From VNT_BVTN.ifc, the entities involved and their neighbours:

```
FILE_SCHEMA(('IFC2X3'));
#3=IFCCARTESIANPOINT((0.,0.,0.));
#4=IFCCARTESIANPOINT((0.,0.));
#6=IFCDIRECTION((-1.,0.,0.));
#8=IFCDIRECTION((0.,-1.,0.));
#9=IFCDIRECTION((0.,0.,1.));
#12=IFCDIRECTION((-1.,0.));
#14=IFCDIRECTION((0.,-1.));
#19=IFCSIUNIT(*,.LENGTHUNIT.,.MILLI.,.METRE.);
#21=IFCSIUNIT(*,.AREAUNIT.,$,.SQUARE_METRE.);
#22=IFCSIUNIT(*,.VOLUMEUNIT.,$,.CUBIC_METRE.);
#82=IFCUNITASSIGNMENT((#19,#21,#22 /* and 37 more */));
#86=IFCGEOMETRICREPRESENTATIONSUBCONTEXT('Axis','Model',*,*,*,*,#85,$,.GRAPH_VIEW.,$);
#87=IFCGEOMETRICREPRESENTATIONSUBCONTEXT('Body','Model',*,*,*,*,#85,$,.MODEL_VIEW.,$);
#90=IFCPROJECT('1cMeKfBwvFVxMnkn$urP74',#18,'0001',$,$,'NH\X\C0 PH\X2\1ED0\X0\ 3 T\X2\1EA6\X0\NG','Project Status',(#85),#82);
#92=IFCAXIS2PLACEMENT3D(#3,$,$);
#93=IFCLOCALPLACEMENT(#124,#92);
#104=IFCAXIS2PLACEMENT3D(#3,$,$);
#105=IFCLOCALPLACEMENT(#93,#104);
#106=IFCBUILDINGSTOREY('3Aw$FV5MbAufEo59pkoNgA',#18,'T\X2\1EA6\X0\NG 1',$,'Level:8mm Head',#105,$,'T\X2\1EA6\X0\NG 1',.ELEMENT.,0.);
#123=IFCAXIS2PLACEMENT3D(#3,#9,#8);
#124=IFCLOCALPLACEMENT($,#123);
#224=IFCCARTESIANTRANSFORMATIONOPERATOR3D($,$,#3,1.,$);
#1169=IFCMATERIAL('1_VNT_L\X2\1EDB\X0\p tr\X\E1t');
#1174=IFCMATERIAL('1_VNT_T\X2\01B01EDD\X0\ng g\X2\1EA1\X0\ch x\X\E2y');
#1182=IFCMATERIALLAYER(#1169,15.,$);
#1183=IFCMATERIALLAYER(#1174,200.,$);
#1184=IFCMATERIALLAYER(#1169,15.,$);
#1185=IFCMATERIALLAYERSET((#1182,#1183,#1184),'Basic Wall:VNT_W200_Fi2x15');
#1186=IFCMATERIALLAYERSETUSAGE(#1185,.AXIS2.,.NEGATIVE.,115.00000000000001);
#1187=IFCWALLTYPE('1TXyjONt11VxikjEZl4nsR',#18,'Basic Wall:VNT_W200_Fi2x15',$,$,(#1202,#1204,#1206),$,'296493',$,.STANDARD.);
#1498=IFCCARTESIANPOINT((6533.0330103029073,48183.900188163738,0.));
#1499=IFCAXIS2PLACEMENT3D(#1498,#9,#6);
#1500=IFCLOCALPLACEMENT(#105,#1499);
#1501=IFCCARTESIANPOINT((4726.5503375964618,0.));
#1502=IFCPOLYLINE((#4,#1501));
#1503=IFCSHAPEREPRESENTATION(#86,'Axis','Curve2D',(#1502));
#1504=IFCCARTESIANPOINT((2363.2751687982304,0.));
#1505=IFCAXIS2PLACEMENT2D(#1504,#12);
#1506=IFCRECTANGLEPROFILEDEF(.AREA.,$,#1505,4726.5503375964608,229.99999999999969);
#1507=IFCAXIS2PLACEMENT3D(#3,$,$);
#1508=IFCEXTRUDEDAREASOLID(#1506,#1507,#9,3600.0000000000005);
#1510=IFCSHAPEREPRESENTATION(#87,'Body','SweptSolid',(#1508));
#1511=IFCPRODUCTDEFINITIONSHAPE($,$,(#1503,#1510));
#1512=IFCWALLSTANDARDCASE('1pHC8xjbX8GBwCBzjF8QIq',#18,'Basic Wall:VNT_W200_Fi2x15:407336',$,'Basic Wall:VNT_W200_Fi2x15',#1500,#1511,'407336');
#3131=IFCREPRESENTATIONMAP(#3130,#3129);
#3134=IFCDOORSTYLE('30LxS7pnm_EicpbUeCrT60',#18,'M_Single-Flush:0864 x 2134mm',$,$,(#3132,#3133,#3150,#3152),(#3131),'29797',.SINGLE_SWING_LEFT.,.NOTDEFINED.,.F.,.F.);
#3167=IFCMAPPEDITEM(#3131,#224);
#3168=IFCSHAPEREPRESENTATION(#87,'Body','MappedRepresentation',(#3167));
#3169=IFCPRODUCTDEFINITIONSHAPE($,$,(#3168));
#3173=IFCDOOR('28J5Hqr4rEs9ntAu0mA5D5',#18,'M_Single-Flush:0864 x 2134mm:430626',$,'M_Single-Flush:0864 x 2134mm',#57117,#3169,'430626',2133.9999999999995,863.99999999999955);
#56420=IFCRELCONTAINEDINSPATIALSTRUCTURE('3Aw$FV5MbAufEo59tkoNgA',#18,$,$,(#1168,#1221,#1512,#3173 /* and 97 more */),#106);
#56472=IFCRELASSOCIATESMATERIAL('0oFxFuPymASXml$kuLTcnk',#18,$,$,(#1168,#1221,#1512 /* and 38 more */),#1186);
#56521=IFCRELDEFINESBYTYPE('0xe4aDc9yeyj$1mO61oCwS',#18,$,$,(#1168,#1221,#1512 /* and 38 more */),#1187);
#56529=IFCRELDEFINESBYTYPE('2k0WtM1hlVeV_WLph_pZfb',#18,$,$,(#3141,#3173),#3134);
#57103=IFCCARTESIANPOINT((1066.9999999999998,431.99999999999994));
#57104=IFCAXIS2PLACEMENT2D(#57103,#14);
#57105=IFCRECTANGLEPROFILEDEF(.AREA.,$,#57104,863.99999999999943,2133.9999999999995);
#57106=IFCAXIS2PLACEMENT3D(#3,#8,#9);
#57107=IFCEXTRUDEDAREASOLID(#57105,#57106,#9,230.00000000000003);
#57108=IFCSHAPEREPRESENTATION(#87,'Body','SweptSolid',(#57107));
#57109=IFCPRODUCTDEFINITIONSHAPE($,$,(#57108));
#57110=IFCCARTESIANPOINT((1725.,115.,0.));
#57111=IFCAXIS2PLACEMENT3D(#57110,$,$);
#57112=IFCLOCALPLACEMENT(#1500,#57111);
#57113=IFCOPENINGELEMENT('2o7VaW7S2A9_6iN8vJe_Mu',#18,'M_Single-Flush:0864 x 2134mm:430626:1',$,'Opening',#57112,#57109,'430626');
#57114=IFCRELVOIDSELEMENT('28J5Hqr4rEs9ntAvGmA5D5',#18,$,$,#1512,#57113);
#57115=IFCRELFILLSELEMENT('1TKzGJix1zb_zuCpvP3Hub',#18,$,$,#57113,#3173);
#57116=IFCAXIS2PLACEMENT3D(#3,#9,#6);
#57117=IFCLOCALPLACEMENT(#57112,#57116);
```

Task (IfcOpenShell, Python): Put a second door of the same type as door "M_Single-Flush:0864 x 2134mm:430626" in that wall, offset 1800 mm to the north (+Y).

```python
import ifcopenshell
import ifcopenshell.api.feature
import ifcopenshell.api.geometry
import ifcopenshell.api.root
import ifcopenshell.geom
import ifcopenshell.util.element
import ifcopenshell.util.placement
import ifcopenshell.util.shape
import ifcopenshell.util.unit

model = ifcopenshell.open("VNT_BVTN.ifc")
unit_scale = ifcopenshell.util.unit.calculate_unit_scale(model)
settings = ifcopenshell.geom.settings()


def volume(element):
    """Net volume in cubic metres, openings subtracted."""
    shape = ifcopenshell.geom.create_shape(settings, element)
    return ifcopenshell.util.shape.get_volume(shape.geometry)


def reuse_history(source, copy):
    """copy_class also copies each property set's owner history, people and application; keep the originals."""
    for rel in copy.IsDefinedBy:
        if rel.is_a("IfcRelDefinesByProperties") and (history := rel.RelatingPropertyDefinition.OwnerHistory):
            rel.RelatingPropertyDefinition.OwnerHistory = source.OwnerHistory
            ifcopenshell.util.element.remove_deep2(model, history)


door = model.by_guid("28J5Hqr4rEs9ntAu0mA5D5")
opening = door.FillsVoids[0].RelatingOpeningElement
wall = opening.VoidsElements[0].RelatingBuildingElement
before = volume(wall)
shift = ifcopenshell.util.placement.get_local_placement(wall.ObjectPlacement)[:3, 0] * 1.8 / unit_scale

# copy_class copies the void relationship, type, container and properties, but no geometry.
new_opening = ifcopenshell.api.root.copy_class(model, product=opening)
new_opening.Representation = ifcopenshell.util.element.copy_deep(
    model, opening.Representation, exclude=["IfcGeometricRepresentationContext", "IfcRepresentationMap"]
)
new_opening.Name = "M_Single-Flush:0864 x 2134mm"
new_opening.Tag = None
new_door = ifcopenshell.api.root.copy_class(model, product=door)
new_door.Representation = ifcopenshell.util.element.copy_deep(
    model, door.Representation, exclude=["IfcGeometricRepresentationContext", "IfcRepresentationMap"]
)
new_door.Name = "M_Single-Flush:0864 x 2134mm"
new_door.Tag = None
reuse_history(door, new_door)
fills = ifcopenshell.api.feature.add_filling(model, opening=new_opening, element=new_door)
fills.OwnerHistory = new_door.OwnerHistory  # required in IFC2X3

for old, new in ((opening, new_opening), (door, new_door)):
    matrix = ifcopenshell.util.placement.get_local_placement(old.ObjectPlacement)
    matrix[:3, 3] += shift
    ifcopenshell.api.geometry.edit_object_placement(model, product=new, matrix=matrix, is_si=False)

after = volume(wall)

print(f"wall volume {before:.3f} -> {after:.3f} m3")

model.write("VNT_BVTN_v2.ifc")
```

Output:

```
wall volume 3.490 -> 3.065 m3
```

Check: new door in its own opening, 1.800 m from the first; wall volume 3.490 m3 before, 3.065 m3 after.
